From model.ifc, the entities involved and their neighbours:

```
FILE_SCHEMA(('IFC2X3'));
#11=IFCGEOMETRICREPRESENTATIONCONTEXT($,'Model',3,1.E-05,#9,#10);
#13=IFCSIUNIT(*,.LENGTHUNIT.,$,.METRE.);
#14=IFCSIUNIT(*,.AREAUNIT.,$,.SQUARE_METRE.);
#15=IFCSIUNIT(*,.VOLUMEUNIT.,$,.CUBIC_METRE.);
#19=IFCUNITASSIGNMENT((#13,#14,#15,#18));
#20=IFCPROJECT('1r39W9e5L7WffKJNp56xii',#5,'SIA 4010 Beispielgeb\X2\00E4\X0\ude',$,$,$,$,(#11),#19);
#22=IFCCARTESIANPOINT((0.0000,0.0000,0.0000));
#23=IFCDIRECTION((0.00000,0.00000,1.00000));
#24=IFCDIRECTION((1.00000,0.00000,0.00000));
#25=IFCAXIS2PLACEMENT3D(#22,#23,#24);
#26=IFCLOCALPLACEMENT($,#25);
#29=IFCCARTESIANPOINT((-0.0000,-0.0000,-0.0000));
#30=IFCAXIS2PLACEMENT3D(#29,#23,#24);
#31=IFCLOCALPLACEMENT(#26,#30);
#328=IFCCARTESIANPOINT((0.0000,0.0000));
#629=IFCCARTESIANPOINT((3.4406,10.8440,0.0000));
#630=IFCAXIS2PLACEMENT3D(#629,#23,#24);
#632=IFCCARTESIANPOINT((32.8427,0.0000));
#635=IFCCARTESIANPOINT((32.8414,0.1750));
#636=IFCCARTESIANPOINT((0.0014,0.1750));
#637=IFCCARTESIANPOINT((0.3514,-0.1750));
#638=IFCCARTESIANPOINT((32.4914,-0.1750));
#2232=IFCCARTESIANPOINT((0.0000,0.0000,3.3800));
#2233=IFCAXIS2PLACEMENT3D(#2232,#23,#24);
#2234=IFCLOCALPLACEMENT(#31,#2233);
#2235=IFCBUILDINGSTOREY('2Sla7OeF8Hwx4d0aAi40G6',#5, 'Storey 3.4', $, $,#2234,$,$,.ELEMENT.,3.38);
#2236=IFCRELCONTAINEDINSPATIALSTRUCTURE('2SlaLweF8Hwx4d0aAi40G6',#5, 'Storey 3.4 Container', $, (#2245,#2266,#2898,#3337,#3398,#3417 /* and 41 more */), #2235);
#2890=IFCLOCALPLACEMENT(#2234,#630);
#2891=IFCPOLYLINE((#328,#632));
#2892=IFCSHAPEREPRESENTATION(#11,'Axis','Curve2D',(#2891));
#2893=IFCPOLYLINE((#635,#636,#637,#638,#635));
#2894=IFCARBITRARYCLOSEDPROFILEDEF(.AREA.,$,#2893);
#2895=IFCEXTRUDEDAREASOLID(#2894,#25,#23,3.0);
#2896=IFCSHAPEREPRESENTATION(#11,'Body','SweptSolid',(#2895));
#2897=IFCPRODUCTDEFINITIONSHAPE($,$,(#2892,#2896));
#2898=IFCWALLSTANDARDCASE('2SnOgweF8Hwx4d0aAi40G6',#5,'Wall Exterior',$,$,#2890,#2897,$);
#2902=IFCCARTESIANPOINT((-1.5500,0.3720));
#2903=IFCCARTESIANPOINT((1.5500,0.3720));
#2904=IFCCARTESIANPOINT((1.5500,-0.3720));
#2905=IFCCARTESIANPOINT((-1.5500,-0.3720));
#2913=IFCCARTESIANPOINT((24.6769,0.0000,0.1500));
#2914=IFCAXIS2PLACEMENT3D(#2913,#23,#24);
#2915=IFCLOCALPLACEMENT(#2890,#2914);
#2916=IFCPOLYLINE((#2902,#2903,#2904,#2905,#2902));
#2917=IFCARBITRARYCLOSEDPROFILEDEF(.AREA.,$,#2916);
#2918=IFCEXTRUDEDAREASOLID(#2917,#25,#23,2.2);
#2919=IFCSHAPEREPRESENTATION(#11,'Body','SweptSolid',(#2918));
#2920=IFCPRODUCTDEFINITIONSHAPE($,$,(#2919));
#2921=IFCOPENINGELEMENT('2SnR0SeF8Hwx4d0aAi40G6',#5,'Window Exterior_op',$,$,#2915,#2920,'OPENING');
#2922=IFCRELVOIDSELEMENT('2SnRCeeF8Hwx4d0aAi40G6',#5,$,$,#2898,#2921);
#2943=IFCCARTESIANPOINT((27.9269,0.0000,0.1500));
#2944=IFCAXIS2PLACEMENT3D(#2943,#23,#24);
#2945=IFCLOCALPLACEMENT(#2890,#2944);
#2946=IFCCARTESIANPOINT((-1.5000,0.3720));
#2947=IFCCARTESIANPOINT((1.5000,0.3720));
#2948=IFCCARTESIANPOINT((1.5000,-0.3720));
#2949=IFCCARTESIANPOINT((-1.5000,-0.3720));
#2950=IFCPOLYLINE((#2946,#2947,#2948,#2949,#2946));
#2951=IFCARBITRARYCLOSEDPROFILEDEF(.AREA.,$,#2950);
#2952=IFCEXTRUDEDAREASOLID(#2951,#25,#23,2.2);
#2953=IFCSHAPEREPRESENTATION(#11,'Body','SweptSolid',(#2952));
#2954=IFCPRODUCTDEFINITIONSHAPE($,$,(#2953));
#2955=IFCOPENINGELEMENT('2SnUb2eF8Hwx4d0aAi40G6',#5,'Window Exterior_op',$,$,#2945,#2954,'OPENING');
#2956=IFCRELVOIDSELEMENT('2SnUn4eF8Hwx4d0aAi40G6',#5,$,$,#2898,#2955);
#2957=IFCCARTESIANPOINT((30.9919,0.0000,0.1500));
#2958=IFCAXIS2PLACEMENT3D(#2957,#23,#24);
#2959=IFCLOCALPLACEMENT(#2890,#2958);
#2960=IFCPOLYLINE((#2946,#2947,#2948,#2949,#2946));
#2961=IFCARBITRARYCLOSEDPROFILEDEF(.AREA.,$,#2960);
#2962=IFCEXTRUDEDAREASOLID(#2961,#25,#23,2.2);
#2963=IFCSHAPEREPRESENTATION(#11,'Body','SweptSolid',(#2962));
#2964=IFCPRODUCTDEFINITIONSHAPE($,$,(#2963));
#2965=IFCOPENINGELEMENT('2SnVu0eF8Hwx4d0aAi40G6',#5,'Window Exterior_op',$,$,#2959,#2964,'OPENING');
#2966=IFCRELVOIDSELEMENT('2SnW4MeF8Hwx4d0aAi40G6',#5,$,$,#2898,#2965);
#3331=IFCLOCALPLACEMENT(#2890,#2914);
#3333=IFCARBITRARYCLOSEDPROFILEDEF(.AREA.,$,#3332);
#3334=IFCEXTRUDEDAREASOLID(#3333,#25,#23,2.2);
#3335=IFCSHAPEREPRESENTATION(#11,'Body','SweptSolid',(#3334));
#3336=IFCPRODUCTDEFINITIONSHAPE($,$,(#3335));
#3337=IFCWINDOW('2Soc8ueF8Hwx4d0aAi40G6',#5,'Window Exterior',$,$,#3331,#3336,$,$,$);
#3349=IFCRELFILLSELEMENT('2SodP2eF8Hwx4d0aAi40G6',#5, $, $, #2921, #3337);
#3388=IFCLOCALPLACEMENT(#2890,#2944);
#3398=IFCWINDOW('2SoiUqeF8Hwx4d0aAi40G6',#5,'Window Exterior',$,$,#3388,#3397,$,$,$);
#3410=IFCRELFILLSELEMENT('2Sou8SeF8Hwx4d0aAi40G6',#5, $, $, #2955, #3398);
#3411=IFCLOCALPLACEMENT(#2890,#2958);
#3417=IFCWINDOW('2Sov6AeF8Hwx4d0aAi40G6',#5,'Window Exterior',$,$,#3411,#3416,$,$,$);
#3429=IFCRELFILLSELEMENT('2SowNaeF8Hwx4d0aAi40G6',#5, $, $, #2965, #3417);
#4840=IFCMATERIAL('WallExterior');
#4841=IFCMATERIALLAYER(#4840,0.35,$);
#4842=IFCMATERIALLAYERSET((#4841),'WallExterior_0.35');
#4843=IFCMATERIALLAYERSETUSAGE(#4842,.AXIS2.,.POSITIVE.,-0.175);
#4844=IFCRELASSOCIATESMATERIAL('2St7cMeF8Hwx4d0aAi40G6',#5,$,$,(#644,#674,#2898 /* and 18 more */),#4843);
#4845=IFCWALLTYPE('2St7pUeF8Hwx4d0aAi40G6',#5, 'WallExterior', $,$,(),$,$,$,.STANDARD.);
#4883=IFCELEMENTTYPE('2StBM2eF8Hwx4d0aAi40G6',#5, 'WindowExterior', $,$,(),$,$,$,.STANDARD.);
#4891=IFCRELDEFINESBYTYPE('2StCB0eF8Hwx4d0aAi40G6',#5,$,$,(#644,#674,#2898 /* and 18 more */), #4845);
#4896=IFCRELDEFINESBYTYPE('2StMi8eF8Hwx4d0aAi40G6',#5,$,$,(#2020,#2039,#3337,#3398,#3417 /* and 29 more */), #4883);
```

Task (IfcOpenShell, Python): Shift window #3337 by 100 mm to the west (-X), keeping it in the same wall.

```python
import ifcopenshell
import ifcopenshell.api.geometry
import ifcopenshell.util.placement
import ifcopenshell.util.unit

model = ifcopenshell.open("model.ifc")
unit_scale = ifcopenshell.util.unit.calculate_unit_scale(model)

window = model.by_id(3337)
opening = window.FillsVoids[0].RelatingOpeningElement
wall = opening.VoidsElements[0].RelatingBuildingElement

wall_matrix = ifcopenshell.util.placement.get_local_placement(wall.ObjectPlacement)
shift = wall_matrix[:3, 0] * -0.1 / unit_scale
before = ifcopenshell.util.placement.get_local_placement(window.ObjectPlacement)[:3, 3].copy()

# The window is not placed relative to its opening, so move both.
for product in (opening, window):
    matrix = ifcopenshell.util.placement.get_local_placement(product.ObjectPlacement)
    matrix[:3, 3] += shift
    ifcopenshell.api.geometry.edit_object_placement(model, product=product, matrix=matrix, is_si=False)

after = ifcopenshell.util.placement.get_local_placement(window.ObjectPlacement)[:3, 3]
print("window moved by", (after - before).round(3) + 0.0)

model.write("model_updated.ifc")
```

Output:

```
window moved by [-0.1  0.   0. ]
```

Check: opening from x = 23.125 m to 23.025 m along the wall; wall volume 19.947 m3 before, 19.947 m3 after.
